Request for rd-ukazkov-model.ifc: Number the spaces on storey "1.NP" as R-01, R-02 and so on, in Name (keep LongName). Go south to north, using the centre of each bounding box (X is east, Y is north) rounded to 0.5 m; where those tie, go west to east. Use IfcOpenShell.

First a look at what the model holds.

```python
import ifcopenshell
import ifcopenshell.util.element
import ifcopenshell.util.placement

model = ifcopenshell.open("rd-ukazkov-model.ifc")
print(model.schema)
storey = next(s for s in model.by_type("IfcBuildingStorey") if s.Name == "1.NP")
spaces = [e for e in ifcopenshell.util.element.get_decomposition(storey) if e.is_a("IfcSpace")]
for e in sorted(spaces, key=lambda e: e.id()):
    origin = ifcopenshell.util.placement.get_local_placement(e.ObjectPlacement)[:3, 3]
    print(e.id(), e.Name, e.LongName, origin.round(2) + 0.0, sep=" | ")
```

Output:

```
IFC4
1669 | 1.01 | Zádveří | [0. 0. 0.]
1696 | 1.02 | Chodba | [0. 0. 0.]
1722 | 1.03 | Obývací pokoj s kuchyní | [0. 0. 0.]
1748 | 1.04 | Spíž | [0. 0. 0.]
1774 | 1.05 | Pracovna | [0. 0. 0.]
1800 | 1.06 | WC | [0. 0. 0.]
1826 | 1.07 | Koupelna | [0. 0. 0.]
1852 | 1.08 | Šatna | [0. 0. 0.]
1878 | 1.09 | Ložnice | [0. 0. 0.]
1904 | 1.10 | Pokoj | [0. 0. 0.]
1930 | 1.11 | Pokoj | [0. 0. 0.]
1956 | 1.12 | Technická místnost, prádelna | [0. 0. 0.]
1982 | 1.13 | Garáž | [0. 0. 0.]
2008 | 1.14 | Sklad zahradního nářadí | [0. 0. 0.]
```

```python
import ifcopenshell
import ifcopenshell.geom
import ifcopenshell.util.element
import ifcopenshell.util.shape

model = ifcopenshell.open("rd-ukazkov-model.ifc")
settings = ifcopenshell.geom.settings()
settings.set("use-world-coords", True)


def centre(element):
    shape = ifcopenshell.geom.create_shape(settings, element)
    return ifcopenshell.util.shape.get_bbox_centroid(shape.geometry)


storey = next(s for s in model.by_type("IfcBuildingStorey") if s.Name == "1.NP")
spaces = [e for e in ifcopenshell.util.element.get_decomposition(storey) if e.is_a("IfcSpace")]

# Insertion points can sit at a corner or the storey origin, so sort by the geometry (in metres).
centres = {e: centre(e) for e in spaces}
spaces.sort(key=lambda e: (round(centres[e][1] / 0.5), centres[e][0]))

for i, e in enumerate(spaces, start=1):
    number = f"R-{i:02d}"
    e.Name = number
    print(e.id(), number)

model.write("rd-ukazkov-model_updated.ifc")
```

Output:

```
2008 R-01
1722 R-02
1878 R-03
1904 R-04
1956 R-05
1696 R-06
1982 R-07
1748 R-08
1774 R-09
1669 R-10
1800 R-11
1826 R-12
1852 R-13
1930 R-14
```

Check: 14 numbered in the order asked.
